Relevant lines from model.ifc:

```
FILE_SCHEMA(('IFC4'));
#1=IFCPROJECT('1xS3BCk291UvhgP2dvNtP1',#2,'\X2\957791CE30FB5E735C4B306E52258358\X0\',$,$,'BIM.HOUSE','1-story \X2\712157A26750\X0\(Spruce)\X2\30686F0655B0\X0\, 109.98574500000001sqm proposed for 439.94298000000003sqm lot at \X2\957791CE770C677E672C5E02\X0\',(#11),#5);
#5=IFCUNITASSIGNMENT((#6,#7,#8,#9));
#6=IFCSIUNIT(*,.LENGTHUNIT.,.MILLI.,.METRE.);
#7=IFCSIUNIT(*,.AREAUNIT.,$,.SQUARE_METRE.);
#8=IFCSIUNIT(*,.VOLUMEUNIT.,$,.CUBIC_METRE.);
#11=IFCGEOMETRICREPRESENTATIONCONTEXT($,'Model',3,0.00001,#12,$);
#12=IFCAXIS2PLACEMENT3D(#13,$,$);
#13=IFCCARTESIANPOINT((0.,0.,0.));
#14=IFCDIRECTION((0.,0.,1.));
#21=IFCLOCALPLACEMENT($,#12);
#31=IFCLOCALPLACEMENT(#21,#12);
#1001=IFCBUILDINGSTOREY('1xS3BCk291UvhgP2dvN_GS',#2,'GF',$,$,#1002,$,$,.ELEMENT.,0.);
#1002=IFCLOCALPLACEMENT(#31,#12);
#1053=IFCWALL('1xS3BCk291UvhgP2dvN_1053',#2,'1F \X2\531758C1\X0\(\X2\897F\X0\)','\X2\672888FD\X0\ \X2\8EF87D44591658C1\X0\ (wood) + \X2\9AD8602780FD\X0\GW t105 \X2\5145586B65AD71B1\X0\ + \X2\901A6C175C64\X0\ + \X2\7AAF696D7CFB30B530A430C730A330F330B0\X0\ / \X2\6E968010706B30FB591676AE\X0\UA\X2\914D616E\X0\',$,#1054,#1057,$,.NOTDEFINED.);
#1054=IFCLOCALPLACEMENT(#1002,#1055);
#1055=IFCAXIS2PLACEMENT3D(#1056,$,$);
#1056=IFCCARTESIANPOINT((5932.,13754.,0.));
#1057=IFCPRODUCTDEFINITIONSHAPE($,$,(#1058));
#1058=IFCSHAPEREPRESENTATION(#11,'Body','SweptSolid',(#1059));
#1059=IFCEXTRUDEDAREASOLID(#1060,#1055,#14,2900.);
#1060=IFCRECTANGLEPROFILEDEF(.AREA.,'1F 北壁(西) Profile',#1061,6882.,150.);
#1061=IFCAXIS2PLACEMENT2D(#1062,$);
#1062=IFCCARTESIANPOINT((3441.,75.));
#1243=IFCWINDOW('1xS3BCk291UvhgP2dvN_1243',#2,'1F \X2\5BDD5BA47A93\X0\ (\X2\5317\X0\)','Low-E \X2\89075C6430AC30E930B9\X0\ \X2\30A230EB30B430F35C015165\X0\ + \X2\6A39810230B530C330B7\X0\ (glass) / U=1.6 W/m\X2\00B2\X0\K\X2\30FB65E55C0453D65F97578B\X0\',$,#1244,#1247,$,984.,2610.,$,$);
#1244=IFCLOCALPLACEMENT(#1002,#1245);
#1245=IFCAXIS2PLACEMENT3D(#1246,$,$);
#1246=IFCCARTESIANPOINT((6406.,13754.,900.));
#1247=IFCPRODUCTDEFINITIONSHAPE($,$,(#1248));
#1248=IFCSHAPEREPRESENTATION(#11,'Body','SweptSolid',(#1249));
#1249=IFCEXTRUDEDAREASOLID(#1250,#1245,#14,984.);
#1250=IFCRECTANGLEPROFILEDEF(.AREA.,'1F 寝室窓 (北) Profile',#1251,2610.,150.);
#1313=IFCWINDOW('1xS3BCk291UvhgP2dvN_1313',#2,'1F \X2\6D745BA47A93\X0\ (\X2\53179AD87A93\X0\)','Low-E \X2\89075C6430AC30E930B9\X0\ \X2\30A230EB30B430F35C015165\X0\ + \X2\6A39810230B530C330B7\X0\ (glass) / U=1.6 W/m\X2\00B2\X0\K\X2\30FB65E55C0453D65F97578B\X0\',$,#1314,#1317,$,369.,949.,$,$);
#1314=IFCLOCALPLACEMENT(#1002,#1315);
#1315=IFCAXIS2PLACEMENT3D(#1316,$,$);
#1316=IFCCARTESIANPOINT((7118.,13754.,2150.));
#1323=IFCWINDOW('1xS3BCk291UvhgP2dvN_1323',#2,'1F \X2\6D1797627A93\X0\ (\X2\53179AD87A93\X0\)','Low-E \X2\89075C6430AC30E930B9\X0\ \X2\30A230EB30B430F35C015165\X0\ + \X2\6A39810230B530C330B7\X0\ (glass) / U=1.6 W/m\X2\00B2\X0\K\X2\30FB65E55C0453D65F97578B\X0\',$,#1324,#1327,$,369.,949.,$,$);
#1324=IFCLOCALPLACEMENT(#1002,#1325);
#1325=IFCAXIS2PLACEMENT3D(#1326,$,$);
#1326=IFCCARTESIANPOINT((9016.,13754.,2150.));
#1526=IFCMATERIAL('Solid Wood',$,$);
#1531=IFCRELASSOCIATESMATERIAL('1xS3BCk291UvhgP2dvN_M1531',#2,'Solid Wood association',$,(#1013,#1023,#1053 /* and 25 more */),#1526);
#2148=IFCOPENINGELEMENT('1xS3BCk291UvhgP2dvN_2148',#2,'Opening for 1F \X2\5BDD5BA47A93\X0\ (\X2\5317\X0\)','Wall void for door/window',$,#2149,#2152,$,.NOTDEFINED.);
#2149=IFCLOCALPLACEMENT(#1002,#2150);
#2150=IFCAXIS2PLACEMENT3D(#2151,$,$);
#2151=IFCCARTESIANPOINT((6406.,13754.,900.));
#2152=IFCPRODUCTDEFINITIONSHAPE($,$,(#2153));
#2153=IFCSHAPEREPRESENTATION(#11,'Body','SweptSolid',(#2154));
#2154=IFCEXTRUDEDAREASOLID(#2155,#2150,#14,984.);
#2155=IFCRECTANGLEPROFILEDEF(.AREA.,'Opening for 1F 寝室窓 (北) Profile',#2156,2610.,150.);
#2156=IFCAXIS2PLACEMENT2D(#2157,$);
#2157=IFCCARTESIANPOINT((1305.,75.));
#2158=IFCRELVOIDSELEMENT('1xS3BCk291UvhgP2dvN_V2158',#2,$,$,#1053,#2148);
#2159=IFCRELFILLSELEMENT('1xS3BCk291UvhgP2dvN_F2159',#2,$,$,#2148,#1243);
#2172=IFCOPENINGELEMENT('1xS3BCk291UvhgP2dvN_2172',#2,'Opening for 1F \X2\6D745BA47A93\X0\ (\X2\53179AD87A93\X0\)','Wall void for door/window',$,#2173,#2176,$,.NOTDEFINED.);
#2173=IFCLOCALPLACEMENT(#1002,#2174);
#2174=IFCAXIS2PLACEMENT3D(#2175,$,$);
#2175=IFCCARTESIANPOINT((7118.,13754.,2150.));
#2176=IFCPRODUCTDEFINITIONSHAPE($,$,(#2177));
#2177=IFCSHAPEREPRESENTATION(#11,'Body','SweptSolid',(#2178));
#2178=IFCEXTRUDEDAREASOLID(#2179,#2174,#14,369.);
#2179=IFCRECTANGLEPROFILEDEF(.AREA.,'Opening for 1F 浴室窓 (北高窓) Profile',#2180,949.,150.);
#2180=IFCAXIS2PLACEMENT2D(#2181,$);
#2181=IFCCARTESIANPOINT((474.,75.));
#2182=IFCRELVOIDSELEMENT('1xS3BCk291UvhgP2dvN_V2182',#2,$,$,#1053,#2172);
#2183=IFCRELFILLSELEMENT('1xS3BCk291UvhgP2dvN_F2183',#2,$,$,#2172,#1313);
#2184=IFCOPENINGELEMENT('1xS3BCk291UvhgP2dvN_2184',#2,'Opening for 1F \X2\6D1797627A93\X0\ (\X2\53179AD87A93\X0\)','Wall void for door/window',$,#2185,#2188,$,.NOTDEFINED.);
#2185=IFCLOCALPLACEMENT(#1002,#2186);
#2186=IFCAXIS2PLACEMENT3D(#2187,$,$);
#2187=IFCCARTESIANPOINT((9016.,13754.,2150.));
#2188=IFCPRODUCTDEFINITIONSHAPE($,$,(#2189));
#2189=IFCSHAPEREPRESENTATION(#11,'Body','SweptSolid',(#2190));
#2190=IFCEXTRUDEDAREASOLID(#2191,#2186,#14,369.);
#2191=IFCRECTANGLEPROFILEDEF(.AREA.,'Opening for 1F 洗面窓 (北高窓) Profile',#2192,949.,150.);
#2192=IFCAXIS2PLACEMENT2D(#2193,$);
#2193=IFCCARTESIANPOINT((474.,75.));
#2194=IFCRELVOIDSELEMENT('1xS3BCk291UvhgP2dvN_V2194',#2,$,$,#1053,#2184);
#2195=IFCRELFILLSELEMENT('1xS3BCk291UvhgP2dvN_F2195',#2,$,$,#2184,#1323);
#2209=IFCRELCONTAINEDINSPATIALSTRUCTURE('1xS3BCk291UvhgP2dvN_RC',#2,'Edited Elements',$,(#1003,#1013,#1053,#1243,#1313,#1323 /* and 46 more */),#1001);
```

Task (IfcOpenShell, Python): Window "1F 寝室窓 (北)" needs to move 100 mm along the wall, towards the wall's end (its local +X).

```python
import ifcopenshell
import ifcopenshell.api.geometry
import ifcopenshell.util.placement

model = ifcopenshell.open("model.ifc")

window = model.by_guid("1xS3BCk291UvhgP2dvN_1243")
opening = window.FillsVoids[0].RelatingOpeningElement
wall = opening.VoidsElements[0].RelatingBuildingElement

wall_matrix = ifcopenshell.util.placement.get_local_placement(wall.ObjectPlacement)
shift = wall_matrix[:3, 0] * 100.0
before = ifcopenshell.util.placement.get_local_placement(window.ObjectPlacement)[:3, 3].copy()

# The window is not placed relative to its opening, so move both.
for product in (opening, window):
    matrix = ifcopenshell.util.placement.get_local_placement(product.ObjectPlacement)
    matrix[:3, 3] += shift
    ifcopenshell.api.geometry.edit_object_placement(model, product=product, matrix=matrix, is_si=False)

after = ifcopenshell.util.placement.get_local_placement(window.ObjectPlacement)[:3, 3]
print("window moved by", (after - before).round(3) + 0.0)

model.write("model_v2.ifc")
```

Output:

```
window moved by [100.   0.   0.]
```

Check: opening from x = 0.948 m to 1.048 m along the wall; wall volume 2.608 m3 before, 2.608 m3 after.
